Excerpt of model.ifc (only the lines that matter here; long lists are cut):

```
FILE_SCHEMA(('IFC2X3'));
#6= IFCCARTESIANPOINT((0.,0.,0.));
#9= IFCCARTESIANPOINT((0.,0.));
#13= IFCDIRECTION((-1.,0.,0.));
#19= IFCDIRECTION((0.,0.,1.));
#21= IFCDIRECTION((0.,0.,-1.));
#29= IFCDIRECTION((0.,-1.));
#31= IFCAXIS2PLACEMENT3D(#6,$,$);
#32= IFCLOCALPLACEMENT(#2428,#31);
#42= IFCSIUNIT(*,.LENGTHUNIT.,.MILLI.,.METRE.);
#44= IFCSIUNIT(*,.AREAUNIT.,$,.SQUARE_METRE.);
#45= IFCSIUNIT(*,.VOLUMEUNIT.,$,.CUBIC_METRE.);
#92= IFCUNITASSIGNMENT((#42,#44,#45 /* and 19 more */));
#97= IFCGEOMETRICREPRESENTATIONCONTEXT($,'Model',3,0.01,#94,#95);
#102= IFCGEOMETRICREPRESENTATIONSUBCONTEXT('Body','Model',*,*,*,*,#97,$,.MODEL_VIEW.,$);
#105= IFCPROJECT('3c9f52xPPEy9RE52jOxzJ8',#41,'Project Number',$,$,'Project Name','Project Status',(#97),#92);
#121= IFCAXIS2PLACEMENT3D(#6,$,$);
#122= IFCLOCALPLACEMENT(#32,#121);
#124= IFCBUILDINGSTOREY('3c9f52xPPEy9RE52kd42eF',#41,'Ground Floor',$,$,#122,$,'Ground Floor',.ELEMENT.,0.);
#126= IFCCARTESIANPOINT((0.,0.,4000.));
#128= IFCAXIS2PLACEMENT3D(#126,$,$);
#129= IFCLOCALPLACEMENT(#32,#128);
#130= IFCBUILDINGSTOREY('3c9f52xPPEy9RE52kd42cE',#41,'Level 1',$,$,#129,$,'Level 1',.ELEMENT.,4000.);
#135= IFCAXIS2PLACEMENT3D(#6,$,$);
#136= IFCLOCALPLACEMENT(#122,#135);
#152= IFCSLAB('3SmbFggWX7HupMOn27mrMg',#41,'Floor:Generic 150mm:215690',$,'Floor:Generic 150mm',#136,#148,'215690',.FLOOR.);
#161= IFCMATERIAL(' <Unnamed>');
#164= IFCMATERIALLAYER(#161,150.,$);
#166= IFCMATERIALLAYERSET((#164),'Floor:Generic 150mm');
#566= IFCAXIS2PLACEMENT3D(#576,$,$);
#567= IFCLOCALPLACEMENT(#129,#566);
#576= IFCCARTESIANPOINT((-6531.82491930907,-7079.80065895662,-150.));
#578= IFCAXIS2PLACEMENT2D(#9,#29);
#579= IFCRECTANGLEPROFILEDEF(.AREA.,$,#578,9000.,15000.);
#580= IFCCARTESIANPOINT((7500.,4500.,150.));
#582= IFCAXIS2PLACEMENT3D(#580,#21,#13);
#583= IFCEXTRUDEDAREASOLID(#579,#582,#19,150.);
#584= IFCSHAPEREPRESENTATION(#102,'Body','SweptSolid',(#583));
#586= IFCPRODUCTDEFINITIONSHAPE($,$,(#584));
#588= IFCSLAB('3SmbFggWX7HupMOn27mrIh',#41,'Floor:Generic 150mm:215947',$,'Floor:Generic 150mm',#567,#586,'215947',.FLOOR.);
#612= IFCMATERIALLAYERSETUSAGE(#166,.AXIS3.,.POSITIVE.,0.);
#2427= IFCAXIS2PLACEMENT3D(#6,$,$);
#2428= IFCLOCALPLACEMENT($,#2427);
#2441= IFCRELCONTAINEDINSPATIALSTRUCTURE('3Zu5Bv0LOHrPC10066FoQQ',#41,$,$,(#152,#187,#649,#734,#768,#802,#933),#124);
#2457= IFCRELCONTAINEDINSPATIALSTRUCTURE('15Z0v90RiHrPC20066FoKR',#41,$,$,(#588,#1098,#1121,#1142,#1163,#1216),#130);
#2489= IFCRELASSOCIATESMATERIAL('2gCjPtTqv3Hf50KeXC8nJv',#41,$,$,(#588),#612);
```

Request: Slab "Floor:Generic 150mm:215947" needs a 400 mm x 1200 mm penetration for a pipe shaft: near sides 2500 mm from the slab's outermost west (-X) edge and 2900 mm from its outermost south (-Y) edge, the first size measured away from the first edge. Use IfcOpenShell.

```python
import numpy as np
import ifcopenshell
import ifcopenshell.api.feature
import ifcopenshell.api.geometry
import ifcopenshell.api.root
import ifcopenshell.geom
import ifcopenshell.util.placement
import ifcopenshell.util.representation
import ifcopenshell.util.shape
import ifcopenshell.util.unit

model = ifcopenshell.open("model.ifc")
unit_scale = ifcopenshell.util.unit.calculate_unit_scale(model)
settings = ifcopenshell.geom.settings()


def volume(element):
    """Net volume in cubic metres, openings subtracted."""
    shape = ifcopenshell.geom.create_shape(settings, element)
    return ifcopenshell.util.shape.get_volume(shape.geometry)


slab = model.by_id(588)
before = volume(slab)

# Extent in the slab's own axes, in metres. The edges named are its -X and -Y sides.
slab_shape = ifcopenshell.geom.create_shape(settings, slab)
vertices = ifcopenshell.util.shape.get_vertices(slab_shape.geometry)
x_min, y_min, bottom = vertices.min(axis=0)
top = vertices[:, 2].max()

opening = ifcopenshell.api.root.create_entity(model, ifc_class="IfcOpeningElement", name="Pipe shaft opening")
context = ifcopenshell.util.representation.get_context(model, "Model", "Body", "MODEL_VIEW")
width, depth = 0.4, 1.2
outline = [(0.0, 0.0), (width, 0.0), (width, depth), (0.0, depth), (0.0, 0.0)]
# Overshoot both faces by 50 mm so the cut is clean.
shape = ifcopenshell.api.geometry.add_slab_representation(
    model, context=context, depth=top - bottom + 0.1, polyline=outline
)
ifcopenshell.api.geometry.assign_representation(model, product=opening, representation=shape)

matrix = ifcopenshell.util.placement.get_local_placement(slab.ObjectPlacement)
matrix[:, 3] = matrix @ np.append(np.array([x_min + 2.5, y_min + 2.9, bottom - 0.05]) / unit_scale, 1.0)
ifcopenshell.api.geometry.edit_object_placement(model, product=opening, matrix=matrix, is_si=False)
ifcopenshell.api.feature.add_feature(model, feature=opening, element=slab)

after = volume(slab)

print(f"slab volume {before:.3f} -> {after:.3f} m3")

model.write("model_edited.ifc")
```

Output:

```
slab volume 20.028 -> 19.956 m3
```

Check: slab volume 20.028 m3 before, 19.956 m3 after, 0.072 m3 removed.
